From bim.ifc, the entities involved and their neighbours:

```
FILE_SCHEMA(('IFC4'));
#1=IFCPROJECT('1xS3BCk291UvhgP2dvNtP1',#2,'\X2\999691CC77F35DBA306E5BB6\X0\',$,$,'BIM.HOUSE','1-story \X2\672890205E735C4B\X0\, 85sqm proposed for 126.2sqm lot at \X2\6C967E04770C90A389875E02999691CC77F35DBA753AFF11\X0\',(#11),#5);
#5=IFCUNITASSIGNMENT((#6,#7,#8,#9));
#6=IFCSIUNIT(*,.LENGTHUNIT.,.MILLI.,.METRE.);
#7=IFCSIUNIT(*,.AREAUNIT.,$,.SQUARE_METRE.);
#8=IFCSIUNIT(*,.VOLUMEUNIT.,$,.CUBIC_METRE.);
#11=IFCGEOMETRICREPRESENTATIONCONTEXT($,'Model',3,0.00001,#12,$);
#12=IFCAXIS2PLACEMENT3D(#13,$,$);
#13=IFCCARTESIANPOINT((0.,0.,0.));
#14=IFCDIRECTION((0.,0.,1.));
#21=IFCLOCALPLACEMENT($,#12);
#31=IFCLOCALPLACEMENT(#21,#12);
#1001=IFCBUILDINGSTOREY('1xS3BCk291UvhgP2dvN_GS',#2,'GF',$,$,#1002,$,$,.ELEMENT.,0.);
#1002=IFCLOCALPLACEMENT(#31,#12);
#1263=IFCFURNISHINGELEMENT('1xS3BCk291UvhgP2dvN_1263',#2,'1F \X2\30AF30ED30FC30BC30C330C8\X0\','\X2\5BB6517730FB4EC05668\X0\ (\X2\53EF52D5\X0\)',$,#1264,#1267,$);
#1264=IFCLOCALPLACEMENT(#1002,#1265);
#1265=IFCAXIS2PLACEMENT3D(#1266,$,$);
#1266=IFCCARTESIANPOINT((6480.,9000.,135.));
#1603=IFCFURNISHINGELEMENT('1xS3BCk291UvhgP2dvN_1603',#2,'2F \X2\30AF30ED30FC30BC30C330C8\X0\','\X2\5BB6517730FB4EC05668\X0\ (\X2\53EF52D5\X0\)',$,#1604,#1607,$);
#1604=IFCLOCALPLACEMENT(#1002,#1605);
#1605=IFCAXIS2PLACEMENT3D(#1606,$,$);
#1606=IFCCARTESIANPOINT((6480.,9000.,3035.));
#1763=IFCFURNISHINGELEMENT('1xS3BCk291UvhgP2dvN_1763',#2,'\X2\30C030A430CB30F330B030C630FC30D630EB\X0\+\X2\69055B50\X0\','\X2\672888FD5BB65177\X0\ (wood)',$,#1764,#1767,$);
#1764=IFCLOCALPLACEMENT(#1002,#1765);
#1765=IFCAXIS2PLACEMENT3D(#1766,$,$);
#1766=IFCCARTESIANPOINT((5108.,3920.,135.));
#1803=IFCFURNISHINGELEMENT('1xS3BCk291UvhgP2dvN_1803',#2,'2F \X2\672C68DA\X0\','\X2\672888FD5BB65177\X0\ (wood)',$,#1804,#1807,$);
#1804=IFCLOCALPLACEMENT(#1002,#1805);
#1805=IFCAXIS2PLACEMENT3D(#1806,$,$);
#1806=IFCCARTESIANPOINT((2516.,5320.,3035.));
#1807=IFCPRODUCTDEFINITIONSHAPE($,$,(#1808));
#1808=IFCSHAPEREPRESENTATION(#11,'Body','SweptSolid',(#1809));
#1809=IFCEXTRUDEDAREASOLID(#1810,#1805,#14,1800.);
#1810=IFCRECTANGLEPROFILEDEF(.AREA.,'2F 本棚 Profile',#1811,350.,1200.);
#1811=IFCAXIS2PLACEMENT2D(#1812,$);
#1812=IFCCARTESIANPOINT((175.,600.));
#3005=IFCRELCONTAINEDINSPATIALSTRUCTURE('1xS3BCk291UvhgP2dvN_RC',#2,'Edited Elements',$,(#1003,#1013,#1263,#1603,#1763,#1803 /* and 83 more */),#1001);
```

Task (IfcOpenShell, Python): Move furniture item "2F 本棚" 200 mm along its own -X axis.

```python
import ifcopenshell
import ifcopenshell.api.geometry
import ifcopenshell.util.placement
import ifcopenshell.util.unit

model = ifcopenshell.open("bim.ifc")
unit_scale = ifcopenshell.util.unit.calculate_unit_scale(model)

item = model.by_guid("1xS3BCk291UvhgP2dvN_1803")
matrix = ifcopenshell.util.placement.get_local_placement(item.ObjectPlacement)
matrix[:3, 3] -= matrix[:3, 0] * 0.2 / unit_scale
ifcopenshell.api.geometry.edit_object_placement(model, product=item, matrix=matrix, is_si=False)

print(ifcopenshell.util.placement.get_local_placement(item.ObjectPlacement).round(3) + 0.0)

model.write("bim_v2.ifc")
```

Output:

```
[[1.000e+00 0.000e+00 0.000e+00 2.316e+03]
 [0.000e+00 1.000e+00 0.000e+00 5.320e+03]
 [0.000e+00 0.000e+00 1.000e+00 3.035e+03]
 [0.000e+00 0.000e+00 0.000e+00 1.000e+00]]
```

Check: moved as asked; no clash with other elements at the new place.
